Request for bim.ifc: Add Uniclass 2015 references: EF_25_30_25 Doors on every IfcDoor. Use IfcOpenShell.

First a look at what the model holds.

```python
import ifcopenshell

model = ifcopenshell.open("bim.ifc")
print(model.schema)
print("classifications:", [c.Name for c in model.by_type("IfcClassification")])
for ifc_class in ("IfcDoor", "IfcRoof", "IfcStair", "IfcWall", "IfcWindow"):
    print(ifc_class, len(model.by_type(ifc_class)))
```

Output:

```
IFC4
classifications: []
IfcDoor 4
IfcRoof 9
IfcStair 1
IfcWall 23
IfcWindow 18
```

```python
import ifcopenshell
import ifcopenshell.api.classification

model = ifcopenshell.open("bim.ifc")

system = ifcopenshell.api.classification.add_classification(model, classification="Uniclass 2015")

codes = {
    "IfcDoor": ("EF_25_30_25", "Doors"),
}
for ifc_class, (code, name) in codes.items():
    products = model.by_type(ifc_class)
    ifcopenshell.api.classification.add_reference(
        model, products=products, classification=system, identification=code, name=name
    )
    print(code, len(products))

model.write("bim_rev.ifc")
```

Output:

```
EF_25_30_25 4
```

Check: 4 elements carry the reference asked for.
